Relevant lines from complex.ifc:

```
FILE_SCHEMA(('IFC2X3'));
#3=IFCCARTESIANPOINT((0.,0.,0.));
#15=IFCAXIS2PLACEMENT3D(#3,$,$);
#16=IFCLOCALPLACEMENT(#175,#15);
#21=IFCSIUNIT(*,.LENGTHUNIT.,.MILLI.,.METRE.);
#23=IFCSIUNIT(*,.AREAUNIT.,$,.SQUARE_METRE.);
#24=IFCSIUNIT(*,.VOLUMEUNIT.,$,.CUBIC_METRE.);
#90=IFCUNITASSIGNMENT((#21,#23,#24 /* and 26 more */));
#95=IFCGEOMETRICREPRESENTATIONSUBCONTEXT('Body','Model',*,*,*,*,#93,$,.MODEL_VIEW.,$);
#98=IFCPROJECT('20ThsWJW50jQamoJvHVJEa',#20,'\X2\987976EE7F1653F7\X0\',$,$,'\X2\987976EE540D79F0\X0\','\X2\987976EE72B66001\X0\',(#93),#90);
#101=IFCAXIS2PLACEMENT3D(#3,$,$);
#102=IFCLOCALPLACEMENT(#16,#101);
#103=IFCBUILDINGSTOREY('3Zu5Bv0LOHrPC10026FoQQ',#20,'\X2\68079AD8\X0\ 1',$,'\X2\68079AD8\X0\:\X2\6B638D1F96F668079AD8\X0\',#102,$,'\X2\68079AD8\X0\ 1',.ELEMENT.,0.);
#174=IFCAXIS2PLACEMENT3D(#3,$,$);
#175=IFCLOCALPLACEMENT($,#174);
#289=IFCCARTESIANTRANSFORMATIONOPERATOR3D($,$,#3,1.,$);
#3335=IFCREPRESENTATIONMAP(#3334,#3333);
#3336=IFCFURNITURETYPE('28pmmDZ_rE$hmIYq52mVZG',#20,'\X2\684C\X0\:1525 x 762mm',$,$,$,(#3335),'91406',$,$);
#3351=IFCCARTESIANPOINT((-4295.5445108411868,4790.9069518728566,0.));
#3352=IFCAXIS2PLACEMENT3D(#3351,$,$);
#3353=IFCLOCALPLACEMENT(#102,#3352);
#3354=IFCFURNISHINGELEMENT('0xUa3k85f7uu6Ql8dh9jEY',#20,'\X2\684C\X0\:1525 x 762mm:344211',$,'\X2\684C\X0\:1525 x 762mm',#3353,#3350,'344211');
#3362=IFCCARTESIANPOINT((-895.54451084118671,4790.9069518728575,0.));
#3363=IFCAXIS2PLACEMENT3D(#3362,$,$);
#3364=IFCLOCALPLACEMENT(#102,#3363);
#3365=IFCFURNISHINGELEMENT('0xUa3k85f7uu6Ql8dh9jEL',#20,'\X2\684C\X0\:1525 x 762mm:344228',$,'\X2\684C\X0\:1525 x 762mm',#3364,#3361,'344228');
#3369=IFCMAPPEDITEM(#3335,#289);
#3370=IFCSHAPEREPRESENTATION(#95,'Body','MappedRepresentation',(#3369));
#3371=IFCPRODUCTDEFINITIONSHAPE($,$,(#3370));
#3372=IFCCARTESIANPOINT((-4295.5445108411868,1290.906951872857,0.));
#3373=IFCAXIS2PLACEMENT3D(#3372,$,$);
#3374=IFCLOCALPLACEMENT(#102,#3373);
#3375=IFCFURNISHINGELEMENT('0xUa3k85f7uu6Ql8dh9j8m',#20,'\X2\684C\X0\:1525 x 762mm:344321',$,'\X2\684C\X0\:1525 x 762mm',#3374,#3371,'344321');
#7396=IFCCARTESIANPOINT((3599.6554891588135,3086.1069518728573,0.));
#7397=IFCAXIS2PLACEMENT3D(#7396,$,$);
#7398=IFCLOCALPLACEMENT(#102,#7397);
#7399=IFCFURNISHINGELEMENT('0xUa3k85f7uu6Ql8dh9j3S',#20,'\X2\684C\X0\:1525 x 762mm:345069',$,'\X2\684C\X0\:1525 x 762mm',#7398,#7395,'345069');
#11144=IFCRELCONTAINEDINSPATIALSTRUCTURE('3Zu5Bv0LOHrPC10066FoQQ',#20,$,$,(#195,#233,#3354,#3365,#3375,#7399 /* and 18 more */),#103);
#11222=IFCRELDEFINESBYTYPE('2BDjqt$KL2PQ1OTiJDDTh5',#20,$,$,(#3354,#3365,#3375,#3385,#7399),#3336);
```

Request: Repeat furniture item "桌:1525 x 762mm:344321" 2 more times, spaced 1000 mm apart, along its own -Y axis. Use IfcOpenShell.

```python
import ifcopenshell
import ifcopenshell.api.geometry
import ifcopenshell.api.root
import ifcopenshell.util.element
import ifcopenshell.util.placement
import ifcopenshell.util.unit

model = ifcopenshell.open("complex.ifc")
unit_scale = ifcopenshell.util.unit.calculate_unit_scale(model)


def reuse_history(source, copy):
    """copy_class also copies each property set's owner history, people and application; keep the originals."""
    for rel in copy.IsDefinedBy:
        if rel.is_a("IfcRelDefinesByProperties") and (history := rel.RelatingPropertyDefinition.OwnerHistory):
            rel.RelatingPropertyDefinition.OwnerHistory = source.OwnerHistory
            ifcopenshell.util.element.remove_deep2(model, history)


source = model.by_guid("0xUa3k85f7uu6Ql8dh9j8m")
base = ifcopenshell.util.placement.get_local_placement(source.ObjectPlacement)
step = -base[:3, 1] * 1 / unit_scale

for i in range(1, 3):
    copy = ifcopenshell.api.root.copy_class(model, product=source)
    copy.Representation = ifcopenshell.util.element.copy_deep(
        model, source.Representation, exclude=["IfcGeometricRepresentationContext", "IfcRepresentationMap"]
    )
    copy.Name = "桌:1525 x 762mm"
    copy.Tag = None
    reuse_history(source, copy)
    matrix = base.copy()
    matrix[:3, 3] += i * step
    print("added at", matrix[:3, 3].round(3) + 0.0)
    ifcopenshell.api.geometry.edit_object_placement(model, product=copy, matrix=matrix, is_si=False)

model.write("complex_updated.ifc")
```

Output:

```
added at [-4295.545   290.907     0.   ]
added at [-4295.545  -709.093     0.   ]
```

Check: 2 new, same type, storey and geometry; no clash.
